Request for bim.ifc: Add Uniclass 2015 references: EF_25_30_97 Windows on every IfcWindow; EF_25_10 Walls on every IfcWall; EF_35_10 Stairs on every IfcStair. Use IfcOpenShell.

First a look at what the model holds.

```python
import ifcopenshell

model = ifcopenshell.open("bim.ifc")
print(model.schema)
print("classifications:", [c.Name for c in model.by_type("IfcClassification")])
for ifc_class in ("IfcDoor", "IfcRoof", "IfcStair", "IfcWall", "IfcWindow"):
    print(ifc_class, len(model.by_type(ifc_class)))
```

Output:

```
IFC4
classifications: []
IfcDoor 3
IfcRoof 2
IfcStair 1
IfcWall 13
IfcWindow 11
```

```python
import ifcopenshell
import ifcopenshell.api.classification

model = ifcopenshell.open("bim.ifc")

system = ifcopenshell.api.classification.add_classification(model, classification="Uniclass 2015")

codes = {
    "IfcWindow": ("EF_25_30_97", "Windows"),
    "IfcWall": ("EF_25_10", "Walls"),
    "IfcStair": ("EF_35_10", "Stairs"),
}
for ifc_class, (code, name) in codes.items():
    products = model.by_type(ifc_class)
    ifcopenshell.api.classification.add_reference(
        model, products=products, classification=system, identification=code, name=name
    )
    print(code, len(products))

model.write("bim_edited.ifc")
```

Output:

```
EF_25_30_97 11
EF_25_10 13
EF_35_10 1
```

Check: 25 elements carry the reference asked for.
